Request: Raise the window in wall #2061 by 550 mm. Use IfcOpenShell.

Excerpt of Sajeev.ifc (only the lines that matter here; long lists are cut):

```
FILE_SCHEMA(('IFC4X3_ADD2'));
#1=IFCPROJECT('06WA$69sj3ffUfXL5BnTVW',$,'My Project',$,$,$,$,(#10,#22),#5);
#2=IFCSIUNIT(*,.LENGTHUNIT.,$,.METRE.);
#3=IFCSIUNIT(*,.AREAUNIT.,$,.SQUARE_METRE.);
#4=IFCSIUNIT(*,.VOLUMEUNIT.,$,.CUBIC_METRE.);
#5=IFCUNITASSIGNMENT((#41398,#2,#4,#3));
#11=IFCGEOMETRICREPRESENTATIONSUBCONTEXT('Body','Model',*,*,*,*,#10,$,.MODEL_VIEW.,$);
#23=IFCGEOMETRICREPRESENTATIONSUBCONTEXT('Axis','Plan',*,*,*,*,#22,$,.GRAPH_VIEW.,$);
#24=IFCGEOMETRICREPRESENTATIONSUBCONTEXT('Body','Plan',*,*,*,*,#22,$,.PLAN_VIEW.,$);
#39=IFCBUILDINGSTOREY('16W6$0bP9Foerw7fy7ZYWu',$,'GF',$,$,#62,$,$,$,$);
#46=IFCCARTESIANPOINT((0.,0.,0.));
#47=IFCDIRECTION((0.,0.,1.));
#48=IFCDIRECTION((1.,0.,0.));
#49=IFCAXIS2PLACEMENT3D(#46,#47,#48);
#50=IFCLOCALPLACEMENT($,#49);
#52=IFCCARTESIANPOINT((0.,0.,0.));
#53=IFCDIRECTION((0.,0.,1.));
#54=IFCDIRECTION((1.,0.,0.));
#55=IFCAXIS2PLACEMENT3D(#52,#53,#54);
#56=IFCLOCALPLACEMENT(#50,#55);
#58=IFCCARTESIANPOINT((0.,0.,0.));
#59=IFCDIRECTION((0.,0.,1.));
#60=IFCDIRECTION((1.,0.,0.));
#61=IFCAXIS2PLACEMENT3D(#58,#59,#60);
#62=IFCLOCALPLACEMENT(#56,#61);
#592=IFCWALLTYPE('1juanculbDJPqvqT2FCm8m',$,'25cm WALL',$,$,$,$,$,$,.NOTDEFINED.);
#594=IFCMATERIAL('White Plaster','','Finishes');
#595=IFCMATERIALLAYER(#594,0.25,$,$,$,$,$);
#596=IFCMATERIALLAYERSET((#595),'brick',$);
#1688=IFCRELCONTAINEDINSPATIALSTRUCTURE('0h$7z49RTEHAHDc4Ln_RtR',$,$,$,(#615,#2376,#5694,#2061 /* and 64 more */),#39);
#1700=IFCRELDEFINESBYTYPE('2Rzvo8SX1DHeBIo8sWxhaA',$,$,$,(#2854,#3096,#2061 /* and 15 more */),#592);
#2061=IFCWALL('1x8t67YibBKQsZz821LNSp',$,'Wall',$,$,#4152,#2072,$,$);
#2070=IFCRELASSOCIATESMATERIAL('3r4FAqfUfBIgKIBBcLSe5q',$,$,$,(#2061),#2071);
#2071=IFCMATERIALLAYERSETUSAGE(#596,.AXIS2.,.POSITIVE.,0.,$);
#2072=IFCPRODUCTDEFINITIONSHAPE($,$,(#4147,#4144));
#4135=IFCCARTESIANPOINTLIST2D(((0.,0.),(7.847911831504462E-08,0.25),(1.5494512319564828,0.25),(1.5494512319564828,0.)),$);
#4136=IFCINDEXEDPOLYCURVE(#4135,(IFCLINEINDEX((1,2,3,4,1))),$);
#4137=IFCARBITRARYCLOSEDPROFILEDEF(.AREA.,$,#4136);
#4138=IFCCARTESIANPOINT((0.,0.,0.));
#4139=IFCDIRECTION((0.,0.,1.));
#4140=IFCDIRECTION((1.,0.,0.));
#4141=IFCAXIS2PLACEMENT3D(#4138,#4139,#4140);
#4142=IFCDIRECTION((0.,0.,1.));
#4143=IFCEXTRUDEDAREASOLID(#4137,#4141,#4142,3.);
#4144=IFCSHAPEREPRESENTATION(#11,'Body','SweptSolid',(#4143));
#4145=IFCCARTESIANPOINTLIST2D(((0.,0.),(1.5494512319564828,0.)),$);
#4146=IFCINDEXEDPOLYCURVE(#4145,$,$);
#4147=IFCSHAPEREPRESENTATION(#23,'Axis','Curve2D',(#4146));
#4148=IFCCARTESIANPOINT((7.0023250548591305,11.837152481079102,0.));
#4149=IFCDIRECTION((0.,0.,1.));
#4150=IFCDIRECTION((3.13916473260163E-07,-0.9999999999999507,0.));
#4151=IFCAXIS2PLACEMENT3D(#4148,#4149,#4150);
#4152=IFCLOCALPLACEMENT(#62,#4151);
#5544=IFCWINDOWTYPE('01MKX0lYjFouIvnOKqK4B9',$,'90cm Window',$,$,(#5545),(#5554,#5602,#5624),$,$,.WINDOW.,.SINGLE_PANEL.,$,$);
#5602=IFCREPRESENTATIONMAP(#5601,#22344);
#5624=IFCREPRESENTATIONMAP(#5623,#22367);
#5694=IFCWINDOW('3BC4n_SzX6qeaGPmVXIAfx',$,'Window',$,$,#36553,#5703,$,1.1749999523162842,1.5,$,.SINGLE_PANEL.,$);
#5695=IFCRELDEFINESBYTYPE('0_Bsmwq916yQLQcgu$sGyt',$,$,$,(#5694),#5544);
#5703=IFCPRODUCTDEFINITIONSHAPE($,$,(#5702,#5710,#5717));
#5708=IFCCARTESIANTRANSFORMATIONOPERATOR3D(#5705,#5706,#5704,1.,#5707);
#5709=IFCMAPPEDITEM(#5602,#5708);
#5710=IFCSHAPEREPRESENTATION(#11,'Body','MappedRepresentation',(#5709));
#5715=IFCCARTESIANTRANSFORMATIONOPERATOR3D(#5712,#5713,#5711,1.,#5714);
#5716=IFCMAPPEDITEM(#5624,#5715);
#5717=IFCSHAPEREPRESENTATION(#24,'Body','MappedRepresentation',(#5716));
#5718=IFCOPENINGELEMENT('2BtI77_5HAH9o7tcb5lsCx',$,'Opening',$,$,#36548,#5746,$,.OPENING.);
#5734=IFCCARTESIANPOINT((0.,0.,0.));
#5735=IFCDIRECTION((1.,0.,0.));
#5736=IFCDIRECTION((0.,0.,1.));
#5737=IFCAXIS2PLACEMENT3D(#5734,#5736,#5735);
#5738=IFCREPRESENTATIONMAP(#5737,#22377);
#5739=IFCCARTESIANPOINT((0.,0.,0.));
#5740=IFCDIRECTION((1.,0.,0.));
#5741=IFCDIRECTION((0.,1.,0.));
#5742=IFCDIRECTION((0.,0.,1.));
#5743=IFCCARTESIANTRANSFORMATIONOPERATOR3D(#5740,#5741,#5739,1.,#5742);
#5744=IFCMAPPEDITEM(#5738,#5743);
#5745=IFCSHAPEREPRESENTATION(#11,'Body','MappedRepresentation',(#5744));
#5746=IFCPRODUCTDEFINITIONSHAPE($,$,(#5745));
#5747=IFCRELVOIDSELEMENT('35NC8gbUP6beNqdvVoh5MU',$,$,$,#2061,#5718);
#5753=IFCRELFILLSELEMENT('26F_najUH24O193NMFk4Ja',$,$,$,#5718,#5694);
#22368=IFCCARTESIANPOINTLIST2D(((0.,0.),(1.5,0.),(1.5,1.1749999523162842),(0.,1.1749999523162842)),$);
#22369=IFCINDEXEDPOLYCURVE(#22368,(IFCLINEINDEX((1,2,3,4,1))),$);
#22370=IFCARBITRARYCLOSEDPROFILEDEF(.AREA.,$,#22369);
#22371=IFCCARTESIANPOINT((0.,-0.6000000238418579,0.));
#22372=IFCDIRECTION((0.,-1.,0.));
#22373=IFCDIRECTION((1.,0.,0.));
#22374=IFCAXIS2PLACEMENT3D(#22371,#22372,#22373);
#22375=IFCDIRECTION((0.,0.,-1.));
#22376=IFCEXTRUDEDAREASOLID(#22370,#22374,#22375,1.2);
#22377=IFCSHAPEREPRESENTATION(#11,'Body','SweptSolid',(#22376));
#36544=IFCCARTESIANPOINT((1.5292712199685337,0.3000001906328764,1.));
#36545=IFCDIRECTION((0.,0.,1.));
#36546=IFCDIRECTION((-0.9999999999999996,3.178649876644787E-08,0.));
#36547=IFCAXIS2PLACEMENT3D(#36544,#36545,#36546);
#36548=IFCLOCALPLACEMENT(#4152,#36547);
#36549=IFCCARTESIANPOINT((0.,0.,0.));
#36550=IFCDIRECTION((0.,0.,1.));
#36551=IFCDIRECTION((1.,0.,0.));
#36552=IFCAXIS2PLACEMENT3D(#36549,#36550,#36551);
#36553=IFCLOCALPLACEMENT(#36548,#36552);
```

```python
import numpy as np
import ifcopenshell
import ifcopenshell.api.geometry
import ifcopenshell.util.placement
import ifcopenshell.util.unit

model = ifcopenshell.open("Sajeev.ifc")
unit_scale = ifcopenshell.util.unit.calculate_unit_scale(model)

window = model.by_guid("3BC4n_SzX6qeaGPmVXIAfx")
opening = window.FillsVoids[0].RelatingOpeningElement
dz = 0.55 / unit_scale

shift = np.array([0.0, 0.0, dz])
# The window is placed relative to its opening, so it follows when the opening moves.
matrix = ifcopenshell.util.placement.get_local_placement(opening.ObjectPlacement)
matrix[:3, 3] += shift
ifcopenshell.api.geometry.edit_object_placement(
    model, product=opening, matrix=matrix, is_si=False, should_transform_children=True
)

print(f"moved by {dz * unit_scale:+.3f} m")

model.write("Sajeev_updated.ifc")
```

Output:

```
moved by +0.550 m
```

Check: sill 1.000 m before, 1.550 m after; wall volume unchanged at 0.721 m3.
